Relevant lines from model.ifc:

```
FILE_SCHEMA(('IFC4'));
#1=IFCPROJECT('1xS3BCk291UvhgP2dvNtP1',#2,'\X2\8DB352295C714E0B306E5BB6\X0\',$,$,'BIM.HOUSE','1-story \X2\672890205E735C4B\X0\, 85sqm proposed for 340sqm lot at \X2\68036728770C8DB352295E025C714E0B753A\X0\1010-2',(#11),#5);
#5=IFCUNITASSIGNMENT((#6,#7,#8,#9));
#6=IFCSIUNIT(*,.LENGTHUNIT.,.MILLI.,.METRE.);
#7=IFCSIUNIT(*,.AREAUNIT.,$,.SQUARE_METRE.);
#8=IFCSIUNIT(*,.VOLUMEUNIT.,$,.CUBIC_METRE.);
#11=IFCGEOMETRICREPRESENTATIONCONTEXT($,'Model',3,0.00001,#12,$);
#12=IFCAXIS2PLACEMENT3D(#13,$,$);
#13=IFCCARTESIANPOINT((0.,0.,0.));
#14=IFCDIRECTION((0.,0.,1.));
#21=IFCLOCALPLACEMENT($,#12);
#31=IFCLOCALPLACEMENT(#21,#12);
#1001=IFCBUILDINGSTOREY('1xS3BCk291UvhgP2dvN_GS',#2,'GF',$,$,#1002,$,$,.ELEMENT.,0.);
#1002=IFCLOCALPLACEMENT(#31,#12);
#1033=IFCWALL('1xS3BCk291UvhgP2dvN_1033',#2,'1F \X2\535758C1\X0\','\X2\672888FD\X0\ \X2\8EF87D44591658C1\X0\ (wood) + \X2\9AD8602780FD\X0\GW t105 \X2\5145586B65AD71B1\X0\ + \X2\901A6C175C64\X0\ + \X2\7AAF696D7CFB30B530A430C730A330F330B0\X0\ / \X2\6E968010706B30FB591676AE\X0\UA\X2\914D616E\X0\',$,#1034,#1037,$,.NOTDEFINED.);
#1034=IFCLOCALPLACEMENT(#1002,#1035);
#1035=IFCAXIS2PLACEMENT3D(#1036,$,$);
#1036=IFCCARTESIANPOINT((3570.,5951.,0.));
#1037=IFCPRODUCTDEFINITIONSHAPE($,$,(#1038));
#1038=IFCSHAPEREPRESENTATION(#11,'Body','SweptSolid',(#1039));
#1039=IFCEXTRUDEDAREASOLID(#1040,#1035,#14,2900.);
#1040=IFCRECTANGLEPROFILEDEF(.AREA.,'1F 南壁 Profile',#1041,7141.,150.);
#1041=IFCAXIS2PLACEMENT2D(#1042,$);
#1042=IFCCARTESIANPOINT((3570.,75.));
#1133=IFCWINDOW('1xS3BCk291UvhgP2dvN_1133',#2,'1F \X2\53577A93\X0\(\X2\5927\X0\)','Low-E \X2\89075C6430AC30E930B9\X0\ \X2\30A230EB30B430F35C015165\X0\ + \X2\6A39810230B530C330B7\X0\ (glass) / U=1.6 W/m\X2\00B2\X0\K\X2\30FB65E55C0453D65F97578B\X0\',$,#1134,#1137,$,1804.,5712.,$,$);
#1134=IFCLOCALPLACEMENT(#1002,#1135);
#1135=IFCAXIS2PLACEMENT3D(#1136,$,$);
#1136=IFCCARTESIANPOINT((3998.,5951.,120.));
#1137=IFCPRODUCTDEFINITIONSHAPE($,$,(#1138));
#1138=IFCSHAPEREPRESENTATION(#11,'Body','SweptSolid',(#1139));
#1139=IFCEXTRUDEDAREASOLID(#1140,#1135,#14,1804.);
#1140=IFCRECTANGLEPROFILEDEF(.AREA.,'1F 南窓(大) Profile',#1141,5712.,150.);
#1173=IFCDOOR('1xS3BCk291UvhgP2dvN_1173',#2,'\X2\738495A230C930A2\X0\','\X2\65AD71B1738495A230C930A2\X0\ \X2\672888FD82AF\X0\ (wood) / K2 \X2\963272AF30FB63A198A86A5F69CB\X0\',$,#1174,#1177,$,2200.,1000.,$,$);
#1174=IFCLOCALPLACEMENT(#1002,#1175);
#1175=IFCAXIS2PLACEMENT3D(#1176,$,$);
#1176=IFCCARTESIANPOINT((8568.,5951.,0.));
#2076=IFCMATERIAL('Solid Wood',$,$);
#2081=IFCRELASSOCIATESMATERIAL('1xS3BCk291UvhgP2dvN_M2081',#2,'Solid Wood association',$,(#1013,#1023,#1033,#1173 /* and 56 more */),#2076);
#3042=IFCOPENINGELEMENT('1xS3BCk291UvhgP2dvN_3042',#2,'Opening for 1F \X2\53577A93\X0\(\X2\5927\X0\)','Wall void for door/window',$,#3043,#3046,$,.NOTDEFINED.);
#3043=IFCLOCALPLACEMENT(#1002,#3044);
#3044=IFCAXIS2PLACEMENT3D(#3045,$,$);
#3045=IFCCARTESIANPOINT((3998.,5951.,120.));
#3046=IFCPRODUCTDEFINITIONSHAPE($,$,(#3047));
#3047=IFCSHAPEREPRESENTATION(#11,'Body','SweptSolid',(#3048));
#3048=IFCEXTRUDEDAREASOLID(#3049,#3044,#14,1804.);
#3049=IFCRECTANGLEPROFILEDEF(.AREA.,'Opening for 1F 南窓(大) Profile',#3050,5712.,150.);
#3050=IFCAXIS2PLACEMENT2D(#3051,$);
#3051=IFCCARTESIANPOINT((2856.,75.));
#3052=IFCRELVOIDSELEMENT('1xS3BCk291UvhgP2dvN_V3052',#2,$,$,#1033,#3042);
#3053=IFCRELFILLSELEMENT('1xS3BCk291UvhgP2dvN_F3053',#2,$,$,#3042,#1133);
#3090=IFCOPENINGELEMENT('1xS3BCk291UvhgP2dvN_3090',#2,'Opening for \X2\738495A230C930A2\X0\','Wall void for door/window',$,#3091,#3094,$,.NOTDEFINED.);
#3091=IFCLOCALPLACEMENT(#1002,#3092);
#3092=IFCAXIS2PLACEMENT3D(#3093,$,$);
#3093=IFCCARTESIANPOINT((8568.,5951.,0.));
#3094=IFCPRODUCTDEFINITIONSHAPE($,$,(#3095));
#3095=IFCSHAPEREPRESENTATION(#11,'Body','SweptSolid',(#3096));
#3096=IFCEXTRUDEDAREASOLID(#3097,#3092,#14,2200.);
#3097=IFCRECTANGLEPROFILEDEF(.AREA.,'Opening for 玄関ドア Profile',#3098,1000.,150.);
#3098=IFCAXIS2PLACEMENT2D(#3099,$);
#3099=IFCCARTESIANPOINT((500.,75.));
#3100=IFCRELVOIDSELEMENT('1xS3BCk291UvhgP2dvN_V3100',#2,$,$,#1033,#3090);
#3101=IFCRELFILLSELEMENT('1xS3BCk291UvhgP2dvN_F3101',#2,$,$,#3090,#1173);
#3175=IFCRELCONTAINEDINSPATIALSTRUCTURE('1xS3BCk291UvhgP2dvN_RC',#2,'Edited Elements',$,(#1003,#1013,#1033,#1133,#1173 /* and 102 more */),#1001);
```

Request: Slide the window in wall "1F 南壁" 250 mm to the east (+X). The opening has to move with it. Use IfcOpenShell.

```python
import ifcopenshell
import ifcopenshell.api.geometry
import ifcopenshell.util.placement

model = ifcopenshell.open("model.ifc")

window = model.by_id(1133)
opening = window.FillsVoids[0].RelatingOpeningElement
wall = opening.VoidsElements[0].RelatingBuildingElement

wall_matrix = ifcopenshell.util.placement.get_local_placement(wall.ObjectPlacement)
shift = wall_matrix[:3, 0] * 250.0
before = ifcopenshell.util.placement.get_local_placement(window.ObjectPlacement)[:3, 3].copy()

# The window is not placed relative to its opening, so move both.
for product in (opening, window):
    matrix = ifcopenshell.util.placement.get_local_placement(product.ObjectPlacement)
    matrix[:3, 3] += shift
    ifcopenshell.api.geometry.edit_object_placement(model, product=product, matrix=matrix, is_si=False)

after = ifcopenshell.util.placement.get_local_placement(window.ObjectPlacement)[:3, 3]
print("window moved by", (after - before).round(3) + 0.0)

model.write("model_edited.ifc")
```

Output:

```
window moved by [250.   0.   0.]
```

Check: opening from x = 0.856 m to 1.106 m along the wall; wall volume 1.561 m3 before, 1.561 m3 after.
